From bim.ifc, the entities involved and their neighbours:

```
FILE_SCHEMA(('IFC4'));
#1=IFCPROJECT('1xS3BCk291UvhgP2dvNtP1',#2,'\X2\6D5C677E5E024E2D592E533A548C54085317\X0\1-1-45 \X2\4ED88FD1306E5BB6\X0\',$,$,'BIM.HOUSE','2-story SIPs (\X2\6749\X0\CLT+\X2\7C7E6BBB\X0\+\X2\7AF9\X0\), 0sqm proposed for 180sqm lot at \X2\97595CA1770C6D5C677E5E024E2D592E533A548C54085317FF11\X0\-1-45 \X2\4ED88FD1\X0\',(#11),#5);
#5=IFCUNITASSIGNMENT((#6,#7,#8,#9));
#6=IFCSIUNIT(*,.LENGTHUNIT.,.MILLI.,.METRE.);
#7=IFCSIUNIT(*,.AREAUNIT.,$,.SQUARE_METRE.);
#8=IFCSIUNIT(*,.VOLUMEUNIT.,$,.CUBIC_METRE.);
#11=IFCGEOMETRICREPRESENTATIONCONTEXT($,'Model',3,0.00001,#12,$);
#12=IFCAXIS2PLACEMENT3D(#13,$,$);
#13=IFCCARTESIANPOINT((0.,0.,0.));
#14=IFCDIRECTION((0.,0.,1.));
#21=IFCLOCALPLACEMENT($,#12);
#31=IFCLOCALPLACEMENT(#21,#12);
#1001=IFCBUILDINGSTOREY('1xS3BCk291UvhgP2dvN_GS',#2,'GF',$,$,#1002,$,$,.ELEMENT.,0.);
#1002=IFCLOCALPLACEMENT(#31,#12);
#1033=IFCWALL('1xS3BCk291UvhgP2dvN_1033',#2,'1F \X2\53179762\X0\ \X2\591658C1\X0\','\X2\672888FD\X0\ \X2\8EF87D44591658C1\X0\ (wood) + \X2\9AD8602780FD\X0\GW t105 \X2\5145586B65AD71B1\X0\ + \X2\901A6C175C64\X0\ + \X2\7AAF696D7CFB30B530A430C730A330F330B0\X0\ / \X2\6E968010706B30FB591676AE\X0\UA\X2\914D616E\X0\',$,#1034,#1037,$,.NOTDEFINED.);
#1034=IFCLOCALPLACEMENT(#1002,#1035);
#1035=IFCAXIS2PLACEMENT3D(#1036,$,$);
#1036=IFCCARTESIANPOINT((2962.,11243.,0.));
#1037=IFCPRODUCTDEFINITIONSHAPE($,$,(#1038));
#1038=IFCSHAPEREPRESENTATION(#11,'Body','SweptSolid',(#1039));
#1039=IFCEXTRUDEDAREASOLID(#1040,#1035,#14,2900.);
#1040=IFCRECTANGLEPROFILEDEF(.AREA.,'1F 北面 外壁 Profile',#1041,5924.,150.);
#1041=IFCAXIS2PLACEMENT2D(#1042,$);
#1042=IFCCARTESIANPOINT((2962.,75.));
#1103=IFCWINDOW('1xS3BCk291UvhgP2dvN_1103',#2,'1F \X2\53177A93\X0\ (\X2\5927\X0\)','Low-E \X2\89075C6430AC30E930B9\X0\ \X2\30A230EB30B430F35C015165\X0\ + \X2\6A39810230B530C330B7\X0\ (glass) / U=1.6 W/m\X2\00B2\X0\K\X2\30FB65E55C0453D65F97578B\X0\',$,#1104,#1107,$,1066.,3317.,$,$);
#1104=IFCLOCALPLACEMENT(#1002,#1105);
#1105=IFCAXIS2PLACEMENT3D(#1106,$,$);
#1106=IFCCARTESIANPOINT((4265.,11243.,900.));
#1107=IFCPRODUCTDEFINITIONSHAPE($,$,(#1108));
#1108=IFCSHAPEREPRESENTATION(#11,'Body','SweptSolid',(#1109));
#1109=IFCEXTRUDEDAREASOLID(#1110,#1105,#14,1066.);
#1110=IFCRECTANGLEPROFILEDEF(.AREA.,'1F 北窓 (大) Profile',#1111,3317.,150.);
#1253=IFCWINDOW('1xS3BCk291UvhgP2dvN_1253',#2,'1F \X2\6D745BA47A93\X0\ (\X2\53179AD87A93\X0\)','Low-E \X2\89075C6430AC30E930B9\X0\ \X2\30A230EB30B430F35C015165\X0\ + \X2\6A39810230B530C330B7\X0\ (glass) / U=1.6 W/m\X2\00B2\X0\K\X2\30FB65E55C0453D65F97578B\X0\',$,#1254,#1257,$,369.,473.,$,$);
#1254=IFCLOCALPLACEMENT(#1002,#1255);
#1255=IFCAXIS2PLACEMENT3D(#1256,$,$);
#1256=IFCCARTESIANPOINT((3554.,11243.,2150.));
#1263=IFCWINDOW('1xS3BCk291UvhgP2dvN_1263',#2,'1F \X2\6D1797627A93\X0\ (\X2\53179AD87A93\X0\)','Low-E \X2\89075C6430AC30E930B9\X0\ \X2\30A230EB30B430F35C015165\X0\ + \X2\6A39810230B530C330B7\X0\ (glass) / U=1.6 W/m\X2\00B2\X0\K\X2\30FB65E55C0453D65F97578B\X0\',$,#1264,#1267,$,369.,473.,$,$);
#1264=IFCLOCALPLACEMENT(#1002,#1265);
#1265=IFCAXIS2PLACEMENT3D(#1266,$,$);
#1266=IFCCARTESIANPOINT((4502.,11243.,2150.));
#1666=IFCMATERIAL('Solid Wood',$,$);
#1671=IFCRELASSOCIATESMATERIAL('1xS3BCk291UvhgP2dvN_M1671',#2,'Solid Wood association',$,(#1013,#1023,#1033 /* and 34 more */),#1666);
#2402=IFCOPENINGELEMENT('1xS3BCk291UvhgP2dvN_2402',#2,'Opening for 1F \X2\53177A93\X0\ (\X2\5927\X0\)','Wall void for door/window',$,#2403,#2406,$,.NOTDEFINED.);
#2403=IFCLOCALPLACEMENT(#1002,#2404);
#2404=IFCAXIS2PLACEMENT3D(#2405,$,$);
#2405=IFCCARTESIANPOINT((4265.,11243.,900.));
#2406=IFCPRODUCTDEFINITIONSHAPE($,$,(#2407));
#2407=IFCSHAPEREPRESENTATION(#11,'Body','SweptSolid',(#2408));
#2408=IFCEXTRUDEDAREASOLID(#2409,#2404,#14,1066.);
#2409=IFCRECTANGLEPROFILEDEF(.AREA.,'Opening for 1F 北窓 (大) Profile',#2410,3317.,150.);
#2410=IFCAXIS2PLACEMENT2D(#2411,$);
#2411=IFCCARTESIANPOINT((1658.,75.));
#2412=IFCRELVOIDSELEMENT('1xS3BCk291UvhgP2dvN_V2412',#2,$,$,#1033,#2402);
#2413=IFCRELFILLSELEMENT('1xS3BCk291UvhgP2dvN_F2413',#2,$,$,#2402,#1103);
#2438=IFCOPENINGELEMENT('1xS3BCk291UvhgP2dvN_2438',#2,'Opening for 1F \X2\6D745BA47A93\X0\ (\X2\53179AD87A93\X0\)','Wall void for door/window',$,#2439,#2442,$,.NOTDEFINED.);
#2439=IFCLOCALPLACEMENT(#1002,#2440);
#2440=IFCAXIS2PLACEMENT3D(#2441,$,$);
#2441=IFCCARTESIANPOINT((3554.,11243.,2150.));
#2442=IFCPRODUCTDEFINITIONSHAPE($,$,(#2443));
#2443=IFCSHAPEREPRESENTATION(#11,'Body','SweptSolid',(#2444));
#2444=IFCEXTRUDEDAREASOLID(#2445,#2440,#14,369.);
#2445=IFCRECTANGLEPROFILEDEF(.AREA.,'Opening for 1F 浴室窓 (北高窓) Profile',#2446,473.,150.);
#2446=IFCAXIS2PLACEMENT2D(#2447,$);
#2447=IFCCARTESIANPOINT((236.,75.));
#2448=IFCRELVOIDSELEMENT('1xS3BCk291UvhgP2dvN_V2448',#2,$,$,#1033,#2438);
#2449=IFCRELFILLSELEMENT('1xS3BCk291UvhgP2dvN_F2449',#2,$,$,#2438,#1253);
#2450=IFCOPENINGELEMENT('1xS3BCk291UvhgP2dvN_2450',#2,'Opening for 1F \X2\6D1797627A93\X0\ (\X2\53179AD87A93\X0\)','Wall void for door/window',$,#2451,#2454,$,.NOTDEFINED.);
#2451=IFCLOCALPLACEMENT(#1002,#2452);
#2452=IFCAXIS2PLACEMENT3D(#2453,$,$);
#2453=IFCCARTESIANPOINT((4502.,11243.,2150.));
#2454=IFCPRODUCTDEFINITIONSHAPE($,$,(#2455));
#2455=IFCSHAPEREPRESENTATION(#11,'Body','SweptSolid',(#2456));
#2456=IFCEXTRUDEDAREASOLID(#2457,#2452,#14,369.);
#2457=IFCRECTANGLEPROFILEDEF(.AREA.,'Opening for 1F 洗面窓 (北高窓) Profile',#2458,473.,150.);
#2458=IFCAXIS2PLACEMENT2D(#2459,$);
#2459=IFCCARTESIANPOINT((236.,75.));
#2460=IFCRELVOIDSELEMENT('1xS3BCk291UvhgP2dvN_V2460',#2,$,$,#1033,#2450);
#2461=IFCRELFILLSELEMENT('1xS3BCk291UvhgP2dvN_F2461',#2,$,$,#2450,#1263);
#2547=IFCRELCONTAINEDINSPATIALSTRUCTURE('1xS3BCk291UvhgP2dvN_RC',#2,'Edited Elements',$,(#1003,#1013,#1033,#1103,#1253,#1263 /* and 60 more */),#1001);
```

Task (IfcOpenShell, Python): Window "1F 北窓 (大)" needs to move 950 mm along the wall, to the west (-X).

```python
import ifcopenshell
import ifcopenshell.api.geometry
import ifcopenshell.util.placement

model = ifcopenshell.open("bim.ifc")

window = model.by_guid("1xS3BCk291UvhgP2dvN_1103")
opening = window.FillsVoids[0].RelatingOpeningElement
wall = opening.VoidsElements[0].RelatingBuildingElement

wall_matrix = ifcopenshell.util.placement.get_local_placement(wall.ObjectPlacement)
shift = wall_matrix[:3, 0] * -950.0
before = ifcopenshell.util.placement.get_local_placement(window.ObjectPlacement)[:3, 3].copy()

# The window is not placed relative to its opening, so move both.
for product in (opening, window):
    matrix = ifcopenshell.util.placement.get_local_placement(product.ObjectPlacement)
    matrix[:3, 3] += shift
    ifcopenshell.api.geometry.edit_object_placement(model, product=product, matrix=matrix, is_si=False)

after = ifcopenshell.util.placement.get_local_placement(window.ObjectPlacement)[:3, 3]
print("window moved by", (after - before).round(3) + 0.0)

model.write("bim_rev.ifc")
```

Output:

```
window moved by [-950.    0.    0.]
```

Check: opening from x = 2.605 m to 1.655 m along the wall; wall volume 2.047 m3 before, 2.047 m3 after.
